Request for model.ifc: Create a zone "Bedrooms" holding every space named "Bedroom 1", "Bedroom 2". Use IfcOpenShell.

First a look at what the model holds.

```python
import ifcopenshell

model = ifcopenshell.open("model.ifc")
print(model.schema)
seen = {}
for space in model.by_type("IfcSpace"):
    seen[space.LongName] = seen.get(space.LongName, 0) + 1
for name, count in sorted(seen.items(), key=str):
    print(count, "x", name)
print("zones:", [z.Name for z in model.by_type("IfcZone")][:20])
```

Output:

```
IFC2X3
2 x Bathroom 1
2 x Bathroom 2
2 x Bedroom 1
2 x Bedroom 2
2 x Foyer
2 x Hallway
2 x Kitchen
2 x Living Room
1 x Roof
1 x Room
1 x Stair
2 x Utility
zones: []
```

```python
import ifcopenshell
import ifcopenshell.api.group
import ifcopenshell.api.root

model = ifcopenshell.open("model.ifc")

names = {"Bedroom 1", "Bedroom 2"}
spaces = [s for s in model.by_type("IfcSpace") if s.LongName in names]

zone = ifcopenshell.api.root.create_entity(model, ifc_class="IfcZone", name="Bedrooms")
ifcopenshell.api.group.assign_group(model, products=spaces, group=zone)
print(len(spaces), "spaces in", zone.Name)

model.write("model_edited.ifc")
```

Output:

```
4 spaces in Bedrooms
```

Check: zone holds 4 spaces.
